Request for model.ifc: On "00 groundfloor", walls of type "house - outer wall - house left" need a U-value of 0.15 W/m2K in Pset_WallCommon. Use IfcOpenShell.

First a look at what the model holds.

```python
import ifcopenshell
import ifcopenshell.util.element

model = ifcopenshell.open("model.ifc")
print(model.schema)
storey = next(s for s in model.by_type("IfcBuildingStorey") if s.Name == "00 groundfloor")
walls = [e for e in ifcopenshell.util.element.get_decomposition(storey) if e.is_a("IfcWall")]
seen = {}
for e in walls:
    element_type = ifcopenshell.util.element.get_type(e)
    key = (element_type.Name if element_type != e and element_type else None, ifcopenshell.util.element.get_pset(e, "Pset_WallCommon", "ThermalTransmittance"))
    seen[key] = seen.get(key, 0) + 1
for (name, value), count in sorted(seen.items(), key=str):
    print(count, "x", name, "|", value)
```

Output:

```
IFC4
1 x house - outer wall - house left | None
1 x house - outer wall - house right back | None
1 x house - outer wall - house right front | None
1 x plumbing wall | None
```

```python
import ifcopenshell
import ifcopenshell.api.pset
import ifcopenshell.util.element

model = ifcopenshell.open("model.ifc")

storey = next(s for s in model.by_type("IfcBuildingStorey") if s.Name == "00 groundfloor")
walls = [e for e in ifcopenshell.util.element.get_decomposition(storey) if e.is_a("IfcWall")]

count = 0
for e in walls:
    element_type = ifcopenshell.util.element.get_type(e)
    if element_type in (None, e) or element_type.Name != "house - outer wall - house left":
        continue
    # add_pset returns the element's existing set when there is one.
    pset = ifcopenshell.api.pset.add_pset(model, product=e, name="Pset_WallCommon")
    ifcopenshell.api.pset.edit_pset(model, pset=pset, properties={"ThermalTransmittance": 0.15})
    count += 1

print(count, "walls updated")

model.write("model_rev.ifc")
```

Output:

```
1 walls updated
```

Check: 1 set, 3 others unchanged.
